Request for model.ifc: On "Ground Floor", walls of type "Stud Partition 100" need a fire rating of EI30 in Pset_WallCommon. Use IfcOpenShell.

First a look at what the model holds.

```python
import ifcopenshell
import ifcopenshell.util.element

model = ifcopenshell.open("model.ifc")
print(model.schema)
storey = next(s for s in model.by_type("IfcBuildingStorey") if s.Name == "Ground Floor")
walls = [e for e in ifcopenshell.util.element.get_decomposition(storey) if e.is_a("IfcWall")]
seen = {}
for e in walls:
    element_type = ifcopenshell.util.element.get_type(e)
    key = (element_type.Name if element_type != e and element_type else None, ifcopenshell.util.element.get_pset(e, "Pset_WallCommon", "FireRating"))
    seen[key] = seen.get(key, 0) + 1
for (name, value), count in sorted(seen.items(), key=str):
    print(count, "x", name, "|", value)
```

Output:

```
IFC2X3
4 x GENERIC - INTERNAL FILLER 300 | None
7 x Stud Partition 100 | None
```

```python
import ifcopenshell
import ifcopenshell.api.pset
import ifcopenshell.util.element

model = ifcopenshell.open("model.ifc")

storey = next(s for s in model.by_type("IfcBuildingStorey") if s.Name == "Ground Floor")
walls = [e for e in ifcopenshell.util.element.get_decomposition(storey) if e.is_a("IfcWall")]

count = 0
for e in walls:
    element_type = ifcopenshell.util.element.get_type(e)
    if element_type in (None, e) or element_type.Name != "Stud Partition 100":
        continue
    # add_pset returns the element's existing set when there is one.
    pset = ifcopenshell.api.pset.add_pset(model, product=e, name="Pset_WallCommon")
    ifcopenshell.api.pset.edit_pset(model, pset=pset, properties={"FireRating": "EI30"})
    count += 1

print(count, "walls updated")

model.write("model_v2.ifc")
```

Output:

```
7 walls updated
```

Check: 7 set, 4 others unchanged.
